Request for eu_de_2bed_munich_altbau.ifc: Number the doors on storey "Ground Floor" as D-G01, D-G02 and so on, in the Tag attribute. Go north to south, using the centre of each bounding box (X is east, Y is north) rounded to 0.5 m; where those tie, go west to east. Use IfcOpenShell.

First a look at what the model holds.

```python
import ifcopenshell
import ifcopenshell.util.element
import ifcopenshell.util.placement

model = ifcopenshell.open("eu_de_2bed_munich_altbau.ifc")
print(model.schema)
storey = next(s for s in model.by_type("IfcBuildingStorey") if s.Name == "Ground Floor")
doors = [e for e in ifcopenshell.util.element.get_decomposition(storey) if e.is_a("IfcDoor")]
for e in sorted(doors, key=lambda e: e.id()):
    origin = ifcopenshell.util.placement.get_local_placement(e.ObjectPlacement)[:3, 3]
    print(e.id(), e.Tag, e.Name, origin.round(2) + 0.0, sep=" | ")
```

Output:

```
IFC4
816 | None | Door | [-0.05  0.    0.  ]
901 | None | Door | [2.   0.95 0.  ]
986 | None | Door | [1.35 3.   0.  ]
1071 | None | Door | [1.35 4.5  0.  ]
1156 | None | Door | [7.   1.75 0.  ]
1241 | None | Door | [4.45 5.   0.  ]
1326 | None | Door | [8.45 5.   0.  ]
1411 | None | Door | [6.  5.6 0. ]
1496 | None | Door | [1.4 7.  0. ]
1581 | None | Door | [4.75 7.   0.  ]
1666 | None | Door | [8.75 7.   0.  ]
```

```python
import ifcopenshell
import ifcopenshell.geom
import ifcopenshell.util.element
import ifcopenshell.util.shape

model = ifcopenshell.open("eu_de_2bed_munich_altbau.ifc")
settings = ifcopenshell.geom.settings()
settings.set("use-world-coords", True)


def centre(element):
    shape = ifcopenshell.geom.create_shape(settings, element)
    return ifcopenshell.util.shape.get_bbox_centroid(shape.geometry)


storey = next(s for s in model.by_type("IfcBuildingStorey") if s.Name == "Ground Floor")
doors = [e for e in ifcopenshell.util.element.get_decomposition(storey) if e.is_a("IfcDoor")]

# Insertion points can sit at a corner or the storey origin, so sort by the geometry (in metres).
centres = {e: centre(e) for e in doors}
doors.sort(key=lambda e: (-round(centres[e][1] / 0.5), centres[e][0]))

for i, e in enumerate(doors, start=1):
    number = f"D-G{i:02d}"
    e.Tag = number
    print(e.id(), number)

model.write("eu_de_2bed_munich_altbau_v2.ifc")
```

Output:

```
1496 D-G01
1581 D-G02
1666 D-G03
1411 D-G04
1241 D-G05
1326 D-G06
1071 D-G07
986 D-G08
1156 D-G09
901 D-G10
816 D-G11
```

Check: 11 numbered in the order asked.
